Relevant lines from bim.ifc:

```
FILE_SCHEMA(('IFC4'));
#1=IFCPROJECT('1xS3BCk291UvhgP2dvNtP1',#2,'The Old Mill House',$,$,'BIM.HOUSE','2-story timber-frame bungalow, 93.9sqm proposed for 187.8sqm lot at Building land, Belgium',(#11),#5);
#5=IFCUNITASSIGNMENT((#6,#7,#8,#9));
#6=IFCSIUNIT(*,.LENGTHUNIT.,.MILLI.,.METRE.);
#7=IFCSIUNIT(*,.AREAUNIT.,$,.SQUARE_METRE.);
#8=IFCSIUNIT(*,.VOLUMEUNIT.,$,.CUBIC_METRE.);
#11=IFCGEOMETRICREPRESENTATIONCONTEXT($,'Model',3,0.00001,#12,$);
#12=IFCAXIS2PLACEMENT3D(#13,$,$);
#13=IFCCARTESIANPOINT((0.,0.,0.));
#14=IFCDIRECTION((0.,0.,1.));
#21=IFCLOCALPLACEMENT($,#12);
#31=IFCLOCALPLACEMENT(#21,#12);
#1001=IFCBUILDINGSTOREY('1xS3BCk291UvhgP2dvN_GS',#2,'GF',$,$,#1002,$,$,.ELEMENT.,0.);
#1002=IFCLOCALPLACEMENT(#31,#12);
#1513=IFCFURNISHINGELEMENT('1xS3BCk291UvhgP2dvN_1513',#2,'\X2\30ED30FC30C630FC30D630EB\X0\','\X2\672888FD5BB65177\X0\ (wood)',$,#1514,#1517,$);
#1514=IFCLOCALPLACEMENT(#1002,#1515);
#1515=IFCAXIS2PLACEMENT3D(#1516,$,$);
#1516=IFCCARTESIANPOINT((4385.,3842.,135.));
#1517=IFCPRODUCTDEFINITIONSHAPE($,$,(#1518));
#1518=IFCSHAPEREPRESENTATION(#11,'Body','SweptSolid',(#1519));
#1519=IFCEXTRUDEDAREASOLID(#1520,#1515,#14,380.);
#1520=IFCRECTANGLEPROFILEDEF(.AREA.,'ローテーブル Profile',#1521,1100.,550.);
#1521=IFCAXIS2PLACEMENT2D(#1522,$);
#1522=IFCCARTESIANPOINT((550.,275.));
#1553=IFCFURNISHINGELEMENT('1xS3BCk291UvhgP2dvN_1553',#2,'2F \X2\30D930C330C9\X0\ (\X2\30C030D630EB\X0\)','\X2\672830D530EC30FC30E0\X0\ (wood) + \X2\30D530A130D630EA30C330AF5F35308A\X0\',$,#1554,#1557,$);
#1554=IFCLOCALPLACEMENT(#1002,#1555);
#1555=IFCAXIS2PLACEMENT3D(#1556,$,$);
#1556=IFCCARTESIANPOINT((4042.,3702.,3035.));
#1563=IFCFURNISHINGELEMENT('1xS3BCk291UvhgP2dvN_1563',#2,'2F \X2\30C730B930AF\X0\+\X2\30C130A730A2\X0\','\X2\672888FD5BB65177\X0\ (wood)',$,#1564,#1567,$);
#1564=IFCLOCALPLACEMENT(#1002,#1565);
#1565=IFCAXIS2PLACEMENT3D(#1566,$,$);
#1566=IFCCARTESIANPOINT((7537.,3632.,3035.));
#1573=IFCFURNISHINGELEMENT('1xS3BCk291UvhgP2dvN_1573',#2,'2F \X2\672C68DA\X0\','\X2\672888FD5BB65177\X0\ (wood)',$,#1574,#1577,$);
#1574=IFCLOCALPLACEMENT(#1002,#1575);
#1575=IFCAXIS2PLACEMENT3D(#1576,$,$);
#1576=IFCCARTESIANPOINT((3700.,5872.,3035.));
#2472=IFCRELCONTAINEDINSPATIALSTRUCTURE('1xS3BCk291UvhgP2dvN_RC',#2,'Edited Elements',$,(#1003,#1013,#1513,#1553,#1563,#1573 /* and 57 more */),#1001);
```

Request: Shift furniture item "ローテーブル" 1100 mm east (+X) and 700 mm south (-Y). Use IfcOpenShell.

```python
import ifcopenshell
import ifcopenshell.api.geometry
import ifcopenshell.util.placement
import ifcopenshell.util.unit

model = ifcopenshell.open("bim.ifc")
unit_scale = ifcopenshell.util.unit.calculate_unit_scale(model)

item = model.by_guid("1xS3BCk291UvhgP2dvN_1513")
matrix = ifcopenshell.util.placement.get_local_placement(item.ObjectPlacement)
matrix[0, 3] += 1.1 / unit_scale
matrix[1, 3] -= 0.7 / unit_scale
ifcopenshell.api.geometry.edit_object_placement(model, product=item, matrix=matrix, is_si=False)

print(ifcopenshell.util.placement.get_local_placement(item.ObjectPlacement).round(3) + 0.0)

model.write("bim_edited.ifc")
```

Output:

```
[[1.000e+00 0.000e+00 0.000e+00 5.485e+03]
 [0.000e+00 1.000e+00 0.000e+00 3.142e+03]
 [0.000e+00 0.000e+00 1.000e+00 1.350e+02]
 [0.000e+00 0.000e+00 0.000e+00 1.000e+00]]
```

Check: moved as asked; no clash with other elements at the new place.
